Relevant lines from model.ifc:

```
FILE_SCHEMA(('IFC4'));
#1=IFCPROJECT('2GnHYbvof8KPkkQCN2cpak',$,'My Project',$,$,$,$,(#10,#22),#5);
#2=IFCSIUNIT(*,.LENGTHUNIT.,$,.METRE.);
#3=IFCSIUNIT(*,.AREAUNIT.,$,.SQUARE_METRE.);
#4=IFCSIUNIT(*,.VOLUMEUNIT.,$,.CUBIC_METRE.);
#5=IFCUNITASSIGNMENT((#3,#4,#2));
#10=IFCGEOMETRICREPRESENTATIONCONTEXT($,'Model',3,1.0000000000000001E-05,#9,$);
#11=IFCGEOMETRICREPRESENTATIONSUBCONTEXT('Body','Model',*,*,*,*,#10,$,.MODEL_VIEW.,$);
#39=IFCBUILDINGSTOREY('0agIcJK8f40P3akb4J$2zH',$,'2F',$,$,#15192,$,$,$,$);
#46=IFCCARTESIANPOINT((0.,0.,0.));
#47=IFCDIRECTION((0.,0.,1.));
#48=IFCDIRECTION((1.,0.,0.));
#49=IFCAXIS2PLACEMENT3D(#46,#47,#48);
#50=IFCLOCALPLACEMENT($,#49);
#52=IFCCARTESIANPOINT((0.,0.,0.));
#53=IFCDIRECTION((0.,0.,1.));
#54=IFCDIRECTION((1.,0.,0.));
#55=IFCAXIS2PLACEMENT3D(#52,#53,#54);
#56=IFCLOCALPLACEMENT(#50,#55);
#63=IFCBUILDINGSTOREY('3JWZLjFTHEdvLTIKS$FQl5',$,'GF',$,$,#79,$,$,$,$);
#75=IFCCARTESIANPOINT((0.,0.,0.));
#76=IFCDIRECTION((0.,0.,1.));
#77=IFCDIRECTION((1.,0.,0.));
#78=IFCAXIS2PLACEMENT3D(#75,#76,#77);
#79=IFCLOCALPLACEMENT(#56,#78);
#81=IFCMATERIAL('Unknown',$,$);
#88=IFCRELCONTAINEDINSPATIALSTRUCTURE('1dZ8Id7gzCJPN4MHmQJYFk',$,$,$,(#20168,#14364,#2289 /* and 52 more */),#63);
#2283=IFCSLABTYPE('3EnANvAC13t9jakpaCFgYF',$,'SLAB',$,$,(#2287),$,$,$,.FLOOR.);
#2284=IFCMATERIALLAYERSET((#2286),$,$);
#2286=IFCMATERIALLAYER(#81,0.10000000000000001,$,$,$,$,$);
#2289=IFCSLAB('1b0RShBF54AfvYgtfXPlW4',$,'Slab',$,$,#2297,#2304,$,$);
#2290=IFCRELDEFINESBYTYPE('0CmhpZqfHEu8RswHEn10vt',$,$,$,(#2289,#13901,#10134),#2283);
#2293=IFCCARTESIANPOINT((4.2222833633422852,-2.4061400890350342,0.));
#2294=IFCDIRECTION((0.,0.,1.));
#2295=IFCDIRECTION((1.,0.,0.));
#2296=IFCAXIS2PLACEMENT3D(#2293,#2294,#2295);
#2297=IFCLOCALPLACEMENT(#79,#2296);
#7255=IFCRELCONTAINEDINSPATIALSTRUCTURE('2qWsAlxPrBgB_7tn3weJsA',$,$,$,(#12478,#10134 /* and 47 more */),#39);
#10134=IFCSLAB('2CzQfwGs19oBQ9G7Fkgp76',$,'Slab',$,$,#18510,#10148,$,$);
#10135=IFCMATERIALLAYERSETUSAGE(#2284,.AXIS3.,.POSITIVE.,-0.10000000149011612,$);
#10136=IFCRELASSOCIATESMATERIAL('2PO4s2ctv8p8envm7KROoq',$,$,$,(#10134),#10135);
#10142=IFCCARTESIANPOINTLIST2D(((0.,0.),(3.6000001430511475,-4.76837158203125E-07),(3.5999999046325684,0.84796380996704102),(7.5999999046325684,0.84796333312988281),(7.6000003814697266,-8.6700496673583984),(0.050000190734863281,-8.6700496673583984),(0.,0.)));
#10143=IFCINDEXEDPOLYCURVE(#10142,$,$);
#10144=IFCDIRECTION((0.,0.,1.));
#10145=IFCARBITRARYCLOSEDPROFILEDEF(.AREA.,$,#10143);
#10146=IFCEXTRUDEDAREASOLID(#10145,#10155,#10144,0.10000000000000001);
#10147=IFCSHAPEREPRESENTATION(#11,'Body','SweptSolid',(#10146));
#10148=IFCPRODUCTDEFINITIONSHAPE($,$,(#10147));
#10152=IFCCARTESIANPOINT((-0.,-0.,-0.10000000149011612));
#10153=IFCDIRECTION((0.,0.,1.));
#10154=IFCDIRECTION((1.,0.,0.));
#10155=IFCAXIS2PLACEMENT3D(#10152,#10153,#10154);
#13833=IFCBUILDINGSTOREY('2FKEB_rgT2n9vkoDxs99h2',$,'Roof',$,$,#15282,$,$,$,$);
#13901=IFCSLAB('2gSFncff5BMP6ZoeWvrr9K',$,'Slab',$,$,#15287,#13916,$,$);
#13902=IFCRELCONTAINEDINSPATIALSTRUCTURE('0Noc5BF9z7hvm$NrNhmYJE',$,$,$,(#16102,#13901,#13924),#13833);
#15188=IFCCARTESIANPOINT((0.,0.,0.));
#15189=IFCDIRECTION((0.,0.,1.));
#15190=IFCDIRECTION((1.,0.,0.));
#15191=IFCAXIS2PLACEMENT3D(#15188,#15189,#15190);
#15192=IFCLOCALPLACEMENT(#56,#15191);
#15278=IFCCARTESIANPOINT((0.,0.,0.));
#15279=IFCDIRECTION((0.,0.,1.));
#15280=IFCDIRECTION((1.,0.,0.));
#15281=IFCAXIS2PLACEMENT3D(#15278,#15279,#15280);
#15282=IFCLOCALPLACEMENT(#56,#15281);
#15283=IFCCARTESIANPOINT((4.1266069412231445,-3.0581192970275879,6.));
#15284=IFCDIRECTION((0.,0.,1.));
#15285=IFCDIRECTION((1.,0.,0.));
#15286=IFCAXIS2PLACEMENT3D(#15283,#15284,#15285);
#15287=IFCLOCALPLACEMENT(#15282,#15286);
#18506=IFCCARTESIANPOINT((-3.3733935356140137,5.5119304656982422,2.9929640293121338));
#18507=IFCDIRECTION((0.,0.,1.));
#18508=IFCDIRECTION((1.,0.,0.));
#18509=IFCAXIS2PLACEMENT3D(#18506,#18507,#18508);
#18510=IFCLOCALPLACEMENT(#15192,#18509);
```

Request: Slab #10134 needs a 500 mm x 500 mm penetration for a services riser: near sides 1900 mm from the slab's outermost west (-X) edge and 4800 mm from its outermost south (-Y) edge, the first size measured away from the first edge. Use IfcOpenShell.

```python
import numpy as np
import ifcopenshell
import ifcopenshell.api.feature
import ifcopenshell.api.geometry
import ifcopenshell.api.root
import ifcopenshell.geom
import ifcopenshell.util.placement
import ifcopenshell.util.representation
import ifcopenshell.util.shape
import ifcopenshell.util.unit

model = ifcopenshell.open("model.ifc")
unit_scale = ifcopenshell.util.unit.calculate_unit_scale(model)
settings = ifcopenshell.geom.settings()


def volume(element):
    """Net volume in cubic metres, openings subtracted."""
    shape = ifcopenshell.geom.create_shape(settings, element)
    return ifcopenshell.util.shape.get_volume(shape.geometry)


slab = model.by_id(10134)
before = volume(slab)

# Extent in the slab's own axes, in metres. The edges named are its -X and -Y sides.
slab_shape = ifcopenshell.geom.create_shape(settings, slab)
vertices = ifcopenshell.util.shape.get_vertices(slab_shape.geometry)
x_min, y_min, bottom = vertices.min(axis=0)
top = vertices[:, 2].max()

opening = ifcopenshell.api.root.create_entity(model, ifc_class="IfcOpeningElement", name="Services riser opening", predefined_type="OPENING")
context = ifcopenshell.util.representation.get_context(model, "Model", "Body", "MODEL_VIEW")
width, depth = 0.5, 0.5
outline = [(0.0, 0.0), (width, 0.0), (width, depth), (0.0, depth), (0.0, 0.0)]
# Overshoot both faces by 50 mm so the cut is clean.
shape = ifcopenshell.api.geometry.add_slab_representation(
    model, context=context, depth=top - bottom + 0.1, polyline=outline
)
ifcopenshell.api.geometry.assign_representation(model, product=opening, representation=shape)

matrix = ifcopenshell.util.placement.get_local_placement(slab.ObjectPlacement)
matrix[:, 3] = matrix @ np.append(np.array([x_min + 1.9, y_min + 4.8, bottom - 0.05]) / unit_scale, 1.0)
ifcopenshell.api.geometry.edit_object_placement(model, product=opening, matrix=matrix, is_si=False)
ifcopenshell.api.feature.add_feature(model, feature=opening, element=slab)

after = volume(slab)

print(f"slab volume {before:.3f} -> {after:.3f} m3")

model.write("model-out.ifc")
```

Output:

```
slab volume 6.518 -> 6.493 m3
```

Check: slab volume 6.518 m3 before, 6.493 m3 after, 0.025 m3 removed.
